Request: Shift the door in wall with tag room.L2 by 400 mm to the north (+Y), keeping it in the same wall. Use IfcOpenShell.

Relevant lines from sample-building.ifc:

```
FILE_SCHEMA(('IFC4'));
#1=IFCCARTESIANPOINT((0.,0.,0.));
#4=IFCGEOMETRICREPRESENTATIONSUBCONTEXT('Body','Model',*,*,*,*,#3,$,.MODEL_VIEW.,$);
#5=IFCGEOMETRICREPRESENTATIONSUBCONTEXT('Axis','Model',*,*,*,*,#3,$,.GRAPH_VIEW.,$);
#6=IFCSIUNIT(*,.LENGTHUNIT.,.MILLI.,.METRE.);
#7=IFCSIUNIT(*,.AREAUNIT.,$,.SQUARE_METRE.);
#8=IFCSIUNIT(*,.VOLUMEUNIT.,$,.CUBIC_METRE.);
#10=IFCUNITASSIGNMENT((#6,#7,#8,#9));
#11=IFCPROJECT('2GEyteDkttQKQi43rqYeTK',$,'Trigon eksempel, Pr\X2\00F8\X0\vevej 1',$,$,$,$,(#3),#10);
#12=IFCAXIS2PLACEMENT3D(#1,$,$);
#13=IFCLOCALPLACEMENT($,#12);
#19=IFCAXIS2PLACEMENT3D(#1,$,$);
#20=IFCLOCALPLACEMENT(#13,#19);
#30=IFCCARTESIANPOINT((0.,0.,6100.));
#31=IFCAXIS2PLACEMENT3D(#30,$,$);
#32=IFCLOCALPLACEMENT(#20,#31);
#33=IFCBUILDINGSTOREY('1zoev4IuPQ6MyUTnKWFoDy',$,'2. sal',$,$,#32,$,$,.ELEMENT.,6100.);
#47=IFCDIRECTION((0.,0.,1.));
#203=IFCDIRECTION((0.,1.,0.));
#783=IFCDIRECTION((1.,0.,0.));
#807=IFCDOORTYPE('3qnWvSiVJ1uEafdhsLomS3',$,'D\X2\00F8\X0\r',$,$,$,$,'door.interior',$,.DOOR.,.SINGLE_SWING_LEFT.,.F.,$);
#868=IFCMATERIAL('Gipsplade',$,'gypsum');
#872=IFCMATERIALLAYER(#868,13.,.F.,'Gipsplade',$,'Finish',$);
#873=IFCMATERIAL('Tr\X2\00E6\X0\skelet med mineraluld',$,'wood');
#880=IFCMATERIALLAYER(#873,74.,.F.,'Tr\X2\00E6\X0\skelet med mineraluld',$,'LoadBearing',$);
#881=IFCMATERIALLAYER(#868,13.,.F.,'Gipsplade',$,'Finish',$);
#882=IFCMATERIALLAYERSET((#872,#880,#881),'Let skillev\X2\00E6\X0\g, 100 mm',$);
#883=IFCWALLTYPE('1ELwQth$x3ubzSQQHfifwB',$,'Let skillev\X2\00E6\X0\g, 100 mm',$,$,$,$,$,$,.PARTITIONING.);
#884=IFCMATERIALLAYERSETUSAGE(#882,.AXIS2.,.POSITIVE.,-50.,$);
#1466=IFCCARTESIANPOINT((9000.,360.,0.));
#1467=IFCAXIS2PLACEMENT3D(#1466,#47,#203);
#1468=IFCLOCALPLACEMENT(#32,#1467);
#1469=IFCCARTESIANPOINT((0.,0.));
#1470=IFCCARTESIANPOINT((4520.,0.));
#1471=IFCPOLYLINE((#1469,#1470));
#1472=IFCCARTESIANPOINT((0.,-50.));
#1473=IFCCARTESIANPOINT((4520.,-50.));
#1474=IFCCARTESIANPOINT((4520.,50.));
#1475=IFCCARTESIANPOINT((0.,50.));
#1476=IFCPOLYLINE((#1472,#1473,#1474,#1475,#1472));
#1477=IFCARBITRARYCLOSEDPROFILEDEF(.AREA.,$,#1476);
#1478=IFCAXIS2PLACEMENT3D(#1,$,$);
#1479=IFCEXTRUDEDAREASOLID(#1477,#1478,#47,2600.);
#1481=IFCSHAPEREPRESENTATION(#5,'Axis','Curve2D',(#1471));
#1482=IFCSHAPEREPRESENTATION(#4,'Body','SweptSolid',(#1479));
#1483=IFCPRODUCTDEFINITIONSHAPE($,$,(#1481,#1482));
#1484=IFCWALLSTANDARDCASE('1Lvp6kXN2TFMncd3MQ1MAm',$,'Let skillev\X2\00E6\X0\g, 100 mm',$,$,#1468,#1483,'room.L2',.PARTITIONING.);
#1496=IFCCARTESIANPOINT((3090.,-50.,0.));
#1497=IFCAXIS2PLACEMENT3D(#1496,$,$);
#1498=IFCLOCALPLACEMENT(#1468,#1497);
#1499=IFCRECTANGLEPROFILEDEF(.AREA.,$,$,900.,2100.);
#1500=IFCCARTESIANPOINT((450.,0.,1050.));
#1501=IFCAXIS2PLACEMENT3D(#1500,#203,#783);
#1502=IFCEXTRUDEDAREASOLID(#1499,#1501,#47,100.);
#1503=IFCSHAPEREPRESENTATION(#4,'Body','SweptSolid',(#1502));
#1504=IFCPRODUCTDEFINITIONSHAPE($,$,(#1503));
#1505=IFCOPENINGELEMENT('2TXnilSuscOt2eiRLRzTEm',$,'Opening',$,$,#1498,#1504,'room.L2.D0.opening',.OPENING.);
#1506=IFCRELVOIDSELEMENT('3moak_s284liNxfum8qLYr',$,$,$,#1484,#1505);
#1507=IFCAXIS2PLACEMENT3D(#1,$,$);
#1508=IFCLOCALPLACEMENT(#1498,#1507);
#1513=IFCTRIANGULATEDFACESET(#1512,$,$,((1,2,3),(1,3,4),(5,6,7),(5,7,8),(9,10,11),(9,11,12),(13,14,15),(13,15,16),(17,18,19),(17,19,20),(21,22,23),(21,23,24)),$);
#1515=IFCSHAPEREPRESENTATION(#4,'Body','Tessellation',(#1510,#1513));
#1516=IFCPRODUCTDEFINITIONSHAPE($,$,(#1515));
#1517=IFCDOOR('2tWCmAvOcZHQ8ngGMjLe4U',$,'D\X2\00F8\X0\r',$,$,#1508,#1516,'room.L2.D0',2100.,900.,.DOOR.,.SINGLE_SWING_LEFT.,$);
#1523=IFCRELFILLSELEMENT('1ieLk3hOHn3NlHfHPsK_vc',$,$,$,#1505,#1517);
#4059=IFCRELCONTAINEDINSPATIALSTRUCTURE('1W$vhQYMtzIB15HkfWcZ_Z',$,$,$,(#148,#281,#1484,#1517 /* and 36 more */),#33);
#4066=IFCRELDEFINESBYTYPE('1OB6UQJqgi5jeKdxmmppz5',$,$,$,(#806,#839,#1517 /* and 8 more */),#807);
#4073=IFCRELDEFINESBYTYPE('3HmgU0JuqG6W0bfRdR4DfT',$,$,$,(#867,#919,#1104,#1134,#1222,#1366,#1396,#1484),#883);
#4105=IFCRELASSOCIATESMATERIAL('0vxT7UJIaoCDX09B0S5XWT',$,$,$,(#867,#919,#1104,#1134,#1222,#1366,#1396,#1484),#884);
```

```python
import ifcopenshell
import ifcopenshell.api.geometry
import ifcopenshell.util.placement

model = ifcopenshell.open("sample-building.ifc")

door = model.by_id(1517)
opening = door.FillsVoids[0].RelatingOpeningElement
wall = opening.VoidsElements[0].RelatingBuildingElement

wall_matrix = ifcopenshell.util.placement.get_local_placement(wall.ObjectPlacement)
shift = wall_matrix[:3, 0] * 400.0
before = ifcopenshell.util.placement.get_local_placement(door.ObjectPlacement)[:3, 3].copy()

# The door is placed relative to its opening, so it follows when the opening moves.
matrix = ifcopenshell.util.placement.get_local_placement(opening.ObjectPlacement)
matrix[:3, 3] += shift
ifcopenshell.api.geometry.edit_object_placement(
    model, product=opening, matrix=matrix, is_si=False, should_transform_children=True
)

after = ifcopenshell.util.placement.get_local_placement(door.ObjectPlacement)[:3, 3]
print("door moved by", (after - before).round(3) + 0.0)

model.write("sample-building_rev.ifc")
```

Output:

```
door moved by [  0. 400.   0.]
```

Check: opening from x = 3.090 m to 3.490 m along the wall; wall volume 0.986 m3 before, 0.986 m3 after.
